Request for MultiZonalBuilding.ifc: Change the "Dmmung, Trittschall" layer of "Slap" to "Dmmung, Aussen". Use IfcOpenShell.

First a look at what the model holds.

```python
import ifcopenshell
import ifcopenshell.util.element

model = ifcopenshell.open("MultiZonalBuilding.ifc")
print(model.schema)
for layer_set in model.by_type("IfcMaterialLayerSet"):
    if layer_set.LayerSetName == "Slap":
        for layer in layer_set.MaterialLayers:
            print(layer.id(), layer.Material and layer.Material.Name, layer.LayerThickness, sep=" | ")
        print(len(ifcopenshell.util.element.get_elements_by_material(model, layer_set)), "elements and types use it")
print(sorted(m.Name for m in model.by_type("IfcMaterial") if m.Name)[:60])
```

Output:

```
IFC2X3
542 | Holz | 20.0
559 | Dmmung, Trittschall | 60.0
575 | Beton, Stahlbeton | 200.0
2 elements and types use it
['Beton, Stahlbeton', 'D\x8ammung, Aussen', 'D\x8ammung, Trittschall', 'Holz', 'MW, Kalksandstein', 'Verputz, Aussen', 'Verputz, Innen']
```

```python
import ifcopenshell
import ifcopenshell.api.material

model = ifcopenshell.open("MultiZonalBuilding.ifc")

layer_set = next(s for s in model.by_type("IfcMaterialLayerSet") if s.LayerSetName == "Slap")
layer = next(l for l in layer_set.MaterialLayers if l.Material and l.Material.Name == 'D\x8ammung, Trittschall')
material = next(m for m in model.by_type("IfcMaterial") if m.Name == 'D\x8ammung, Aussen')

# Point this one layer at the other material; renaming the old one would change it everywhere.
ifcopenshell.api.material.edit_layer(model, layer=layer, attributes={}, material=material)

print([l.Material.Name if l.Material else None for l in layer_set.MaterialLayers])

model.write("MultiZonalBuilding-out.ifc")
```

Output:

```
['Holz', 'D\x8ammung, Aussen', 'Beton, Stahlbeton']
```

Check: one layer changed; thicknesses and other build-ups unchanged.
